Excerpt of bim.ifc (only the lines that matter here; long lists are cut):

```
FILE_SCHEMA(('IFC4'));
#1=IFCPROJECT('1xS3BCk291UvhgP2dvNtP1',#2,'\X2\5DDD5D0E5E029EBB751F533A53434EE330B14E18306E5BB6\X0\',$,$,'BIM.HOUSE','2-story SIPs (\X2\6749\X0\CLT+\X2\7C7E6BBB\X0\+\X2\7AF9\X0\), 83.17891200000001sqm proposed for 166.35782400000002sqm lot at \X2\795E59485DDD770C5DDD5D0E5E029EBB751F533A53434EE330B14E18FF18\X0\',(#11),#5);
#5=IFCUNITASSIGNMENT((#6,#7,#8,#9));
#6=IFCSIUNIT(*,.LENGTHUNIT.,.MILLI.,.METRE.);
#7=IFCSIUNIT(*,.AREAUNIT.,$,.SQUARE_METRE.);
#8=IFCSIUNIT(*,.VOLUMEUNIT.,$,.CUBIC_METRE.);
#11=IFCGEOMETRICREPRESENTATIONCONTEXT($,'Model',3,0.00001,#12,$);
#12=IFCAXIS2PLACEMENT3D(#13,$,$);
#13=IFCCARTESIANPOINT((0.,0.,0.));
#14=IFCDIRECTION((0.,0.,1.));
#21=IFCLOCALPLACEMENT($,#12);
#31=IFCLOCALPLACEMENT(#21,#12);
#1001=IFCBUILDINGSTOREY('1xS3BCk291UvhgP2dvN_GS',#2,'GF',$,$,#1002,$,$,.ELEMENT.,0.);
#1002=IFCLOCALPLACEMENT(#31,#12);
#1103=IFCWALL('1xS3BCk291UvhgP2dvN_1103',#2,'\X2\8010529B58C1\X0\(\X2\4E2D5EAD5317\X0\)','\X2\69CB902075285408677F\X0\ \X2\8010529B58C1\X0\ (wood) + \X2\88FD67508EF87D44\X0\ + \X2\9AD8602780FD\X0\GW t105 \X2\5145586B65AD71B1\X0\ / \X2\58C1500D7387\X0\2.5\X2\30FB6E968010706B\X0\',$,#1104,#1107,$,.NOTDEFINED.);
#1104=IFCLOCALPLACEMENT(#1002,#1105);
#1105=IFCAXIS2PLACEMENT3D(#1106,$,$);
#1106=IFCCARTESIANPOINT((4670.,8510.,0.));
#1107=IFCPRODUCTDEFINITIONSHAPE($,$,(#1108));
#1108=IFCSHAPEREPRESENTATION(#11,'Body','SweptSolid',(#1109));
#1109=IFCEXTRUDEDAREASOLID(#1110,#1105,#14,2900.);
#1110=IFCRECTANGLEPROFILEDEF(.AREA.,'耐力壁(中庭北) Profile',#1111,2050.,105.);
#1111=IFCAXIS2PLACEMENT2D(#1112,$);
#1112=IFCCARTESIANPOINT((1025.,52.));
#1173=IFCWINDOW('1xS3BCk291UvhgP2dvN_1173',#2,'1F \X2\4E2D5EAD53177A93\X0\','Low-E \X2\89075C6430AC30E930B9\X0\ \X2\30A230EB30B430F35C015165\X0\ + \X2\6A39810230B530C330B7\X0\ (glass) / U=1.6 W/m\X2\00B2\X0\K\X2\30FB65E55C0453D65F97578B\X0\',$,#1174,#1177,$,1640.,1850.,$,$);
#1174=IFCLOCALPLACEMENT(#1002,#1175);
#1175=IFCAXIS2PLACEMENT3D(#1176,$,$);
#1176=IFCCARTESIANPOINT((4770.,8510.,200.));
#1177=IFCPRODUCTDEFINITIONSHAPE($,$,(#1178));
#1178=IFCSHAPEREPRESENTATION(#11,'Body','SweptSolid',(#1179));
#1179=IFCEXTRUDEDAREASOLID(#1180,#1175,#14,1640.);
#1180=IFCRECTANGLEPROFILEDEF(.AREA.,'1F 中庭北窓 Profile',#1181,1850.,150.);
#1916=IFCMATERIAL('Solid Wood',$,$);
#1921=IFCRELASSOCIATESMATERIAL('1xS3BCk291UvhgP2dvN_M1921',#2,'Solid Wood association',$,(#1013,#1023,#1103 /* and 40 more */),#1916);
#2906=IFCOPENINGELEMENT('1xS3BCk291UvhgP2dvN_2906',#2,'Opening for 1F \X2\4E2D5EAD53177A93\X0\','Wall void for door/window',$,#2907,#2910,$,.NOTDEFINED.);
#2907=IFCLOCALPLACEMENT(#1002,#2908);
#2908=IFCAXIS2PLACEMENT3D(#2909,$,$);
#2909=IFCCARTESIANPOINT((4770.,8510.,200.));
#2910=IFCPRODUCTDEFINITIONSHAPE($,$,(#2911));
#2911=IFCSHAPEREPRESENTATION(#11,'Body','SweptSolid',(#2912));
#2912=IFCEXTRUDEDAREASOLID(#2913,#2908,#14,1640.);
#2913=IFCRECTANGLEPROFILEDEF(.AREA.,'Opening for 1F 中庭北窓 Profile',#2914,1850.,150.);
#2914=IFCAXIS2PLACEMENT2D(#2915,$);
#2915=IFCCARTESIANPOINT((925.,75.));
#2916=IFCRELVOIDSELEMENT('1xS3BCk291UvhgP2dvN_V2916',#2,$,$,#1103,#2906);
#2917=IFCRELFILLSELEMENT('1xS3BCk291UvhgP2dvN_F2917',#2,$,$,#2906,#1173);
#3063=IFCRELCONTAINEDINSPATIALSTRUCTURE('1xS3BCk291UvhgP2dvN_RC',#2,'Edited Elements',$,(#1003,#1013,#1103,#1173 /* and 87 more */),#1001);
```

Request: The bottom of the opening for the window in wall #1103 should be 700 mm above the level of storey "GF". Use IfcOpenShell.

```python
import numpy as np
import ifcopenshell
import ifcopenshell.api.geometry
import ifcopenshell.geom
import ifcopenshell.util.element
import ifcopenshell.util.placement
import ifcopenshell.util.shape
import ifcopenshell.util.unit

model = ifcopenshell.open("bim.ifc")
unit_scale = ifcopenshell.util.unit.calculate_unit_scale(model)

window = model.by_guid("1xS3BCk291UvhgP2dvN_1173")
opening = window.FillsVoids[0].RelatingOpeningElement
storey = ifcopenshell.util.element.get_container(window, ifc_class="IfcBuildingStorey")
level = ifcopenshell.util.placement.get_local_placement(storey.ObjectPlacement)[2, 3]

# The opening's origin need not be at the sill, so measure its lowest point.
shape = ifcopenshell.geom.create_shape(ifcopenshell.geom.settings(), opening)
bottom = ifcopenshell.util.shape.get_shape_bottom_elevation(shape, shape.geometry) / unit_scale
dz = level + 0.7 / unit_scale - bottom

shift = np.array([0.0, 0.0, dz])
# The window is not placed relative to its opening, so move both.
for product in (opening, window):
    matrix = ifcopenshell.util.placement.get_local_placement(product.ObjectPlacement)
    matrix[:3, 3] += shift
    ifcopenshell.api.geometry.edit_object_placement(model, product=product, matrix=matrix, is_si=False)

print(f"moved by {dz * unit_scale:+.3f} m")

model.write("bim_edited.ifc")
```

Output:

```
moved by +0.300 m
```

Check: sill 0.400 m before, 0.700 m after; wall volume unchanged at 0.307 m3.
